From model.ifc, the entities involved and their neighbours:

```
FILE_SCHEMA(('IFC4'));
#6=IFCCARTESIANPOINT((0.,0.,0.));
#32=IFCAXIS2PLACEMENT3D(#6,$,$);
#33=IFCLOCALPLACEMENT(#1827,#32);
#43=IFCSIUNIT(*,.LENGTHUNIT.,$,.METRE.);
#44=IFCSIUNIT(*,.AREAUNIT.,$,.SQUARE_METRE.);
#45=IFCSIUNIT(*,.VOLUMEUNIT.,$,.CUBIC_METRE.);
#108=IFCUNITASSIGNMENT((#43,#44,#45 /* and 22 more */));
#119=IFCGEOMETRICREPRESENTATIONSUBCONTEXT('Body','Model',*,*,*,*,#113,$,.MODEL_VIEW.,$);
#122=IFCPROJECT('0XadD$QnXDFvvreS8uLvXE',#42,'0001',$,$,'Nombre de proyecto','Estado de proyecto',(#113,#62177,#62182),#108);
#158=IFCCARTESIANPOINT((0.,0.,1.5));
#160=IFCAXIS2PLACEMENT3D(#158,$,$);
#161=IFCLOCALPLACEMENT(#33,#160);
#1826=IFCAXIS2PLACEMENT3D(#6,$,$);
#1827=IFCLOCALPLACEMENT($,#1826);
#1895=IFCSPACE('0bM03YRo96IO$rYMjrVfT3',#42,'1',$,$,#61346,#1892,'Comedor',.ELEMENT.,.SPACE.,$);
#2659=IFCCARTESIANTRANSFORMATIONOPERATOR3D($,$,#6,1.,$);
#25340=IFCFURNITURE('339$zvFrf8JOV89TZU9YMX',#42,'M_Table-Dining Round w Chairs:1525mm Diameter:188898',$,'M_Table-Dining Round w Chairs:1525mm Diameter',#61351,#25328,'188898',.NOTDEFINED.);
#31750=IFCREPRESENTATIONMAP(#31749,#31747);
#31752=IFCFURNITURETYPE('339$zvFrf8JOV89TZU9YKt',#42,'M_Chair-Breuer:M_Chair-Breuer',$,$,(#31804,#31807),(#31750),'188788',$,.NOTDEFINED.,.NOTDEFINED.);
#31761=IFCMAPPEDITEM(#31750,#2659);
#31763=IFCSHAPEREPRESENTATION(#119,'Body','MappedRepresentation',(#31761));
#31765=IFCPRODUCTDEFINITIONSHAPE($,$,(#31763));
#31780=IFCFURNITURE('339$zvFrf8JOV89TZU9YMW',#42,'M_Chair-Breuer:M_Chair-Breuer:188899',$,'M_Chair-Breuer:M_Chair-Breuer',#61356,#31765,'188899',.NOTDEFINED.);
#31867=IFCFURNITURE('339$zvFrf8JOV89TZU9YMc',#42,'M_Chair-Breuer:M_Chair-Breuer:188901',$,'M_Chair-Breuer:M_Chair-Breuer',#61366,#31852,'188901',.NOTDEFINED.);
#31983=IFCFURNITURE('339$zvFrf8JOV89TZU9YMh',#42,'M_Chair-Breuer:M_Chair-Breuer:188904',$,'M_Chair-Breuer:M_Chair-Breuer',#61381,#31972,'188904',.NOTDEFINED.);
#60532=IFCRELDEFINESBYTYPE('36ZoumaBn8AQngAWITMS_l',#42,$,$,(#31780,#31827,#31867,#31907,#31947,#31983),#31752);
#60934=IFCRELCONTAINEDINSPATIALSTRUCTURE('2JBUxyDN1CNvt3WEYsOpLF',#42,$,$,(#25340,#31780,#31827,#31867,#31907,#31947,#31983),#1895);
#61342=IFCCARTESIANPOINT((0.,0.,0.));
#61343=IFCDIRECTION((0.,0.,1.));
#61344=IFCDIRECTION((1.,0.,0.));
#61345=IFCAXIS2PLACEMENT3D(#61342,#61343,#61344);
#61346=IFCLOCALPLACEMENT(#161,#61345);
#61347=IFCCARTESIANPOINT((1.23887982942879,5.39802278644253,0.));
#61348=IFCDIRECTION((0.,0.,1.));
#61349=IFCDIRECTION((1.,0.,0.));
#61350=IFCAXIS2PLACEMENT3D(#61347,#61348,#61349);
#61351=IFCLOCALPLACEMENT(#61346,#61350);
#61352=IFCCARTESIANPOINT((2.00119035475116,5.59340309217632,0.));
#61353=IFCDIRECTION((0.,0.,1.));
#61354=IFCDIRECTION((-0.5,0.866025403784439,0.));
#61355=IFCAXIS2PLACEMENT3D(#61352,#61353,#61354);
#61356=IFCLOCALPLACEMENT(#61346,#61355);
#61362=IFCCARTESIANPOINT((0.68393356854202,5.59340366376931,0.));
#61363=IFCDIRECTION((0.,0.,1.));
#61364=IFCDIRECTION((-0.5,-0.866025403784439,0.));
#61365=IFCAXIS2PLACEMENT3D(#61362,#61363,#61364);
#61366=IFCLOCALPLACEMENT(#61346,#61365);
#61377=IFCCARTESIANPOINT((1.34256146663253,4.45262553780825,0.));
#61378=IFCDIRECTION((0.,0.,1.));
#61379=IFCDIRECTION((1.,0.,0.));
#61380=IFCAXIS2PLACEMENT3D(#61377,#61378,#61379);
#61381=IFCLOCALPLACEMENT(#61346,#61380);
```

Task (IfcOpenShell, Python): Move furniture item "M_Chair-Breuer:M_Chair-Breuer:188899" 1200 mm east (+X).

```python
import ifcopenshell
import ifcopenshell.api.geometry
import ifcopenshell.util.placement

model = ifcopenshell.open("model.ifc")

item = model.by_guid("339$zvFrf8JOV89TZU9YMW")
matrix = ifcopenshell.util.placement.get_local_placement(item.ObjectPlacement)
matrix[0, 3] += 1.2
ifcopenshell.api.geometry.edit_object_placement(model, product=item, matrix=matrix, is_si=False)

print(ifcopenshell.util.placement.get_local_placement(item.ObjectPlacement).round(3) + 0.0)

model.write("model_rev.ifc")
```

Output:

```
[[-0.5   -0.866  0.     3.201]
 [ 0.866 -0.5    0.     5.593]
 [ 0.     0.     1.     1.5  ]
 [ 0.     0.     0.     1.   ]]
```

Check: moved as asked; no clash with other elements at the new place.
